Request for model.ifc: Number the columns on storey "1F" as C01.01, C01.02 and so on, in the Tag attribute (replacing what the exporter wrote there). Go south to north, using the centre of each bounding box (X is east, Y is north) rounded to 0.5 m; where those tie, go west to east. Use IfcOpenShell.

First a look at what the model holds.

```python
import ifcopenshell
import ifcopenshell.util.element
import ifcopenshell.util.placement

model = ifcopenshell.open("model.ifc")
print(model.schema)
storey = next(s for s in model.by_type("IfcBuildingStorey") if s.Name == "1F")
columns = [e for e in ifcopenshell.util.element.get_decomposition(storey) if e.is_a("IfcColumn")]
for e in sorted(columns, key=lambda e: e.id()):
    origin = ifcopenshell.util.placement.get_local_placement(e.ObjectPlacement)[:3, 3]
    print(e.id(), e.Tag, e.Name, origin.round(2) + 0.0, sep=" | ")
```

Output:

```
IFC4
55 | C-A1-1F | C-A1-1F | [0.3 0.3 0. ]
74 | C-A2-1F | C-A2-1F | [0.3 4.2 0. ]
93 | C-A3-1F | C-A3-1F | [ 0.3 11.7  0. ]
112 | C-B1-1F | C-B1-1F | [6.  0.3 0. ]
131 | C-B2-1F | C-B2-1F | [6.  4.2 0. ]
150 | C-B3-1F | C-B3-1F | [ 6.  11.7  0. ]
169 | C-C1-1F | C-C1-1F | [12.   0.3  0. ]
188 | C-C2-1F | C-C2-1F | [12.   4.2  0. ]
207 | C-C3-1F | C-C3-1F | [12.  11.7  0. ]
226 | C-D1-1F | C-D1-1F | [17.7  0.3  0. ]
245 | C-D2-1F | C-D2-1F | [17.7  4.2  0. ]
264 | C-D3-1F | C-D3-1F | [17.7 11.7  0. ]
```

```python
import ifcopenshell
import ifcopenshell.geom
import ifcopenshell.util.element
import ifcopenshell.util.shape

model = ifcopenshell.open("model.ifc")
settings = ifcopenshell.geom.settings()
settings.set("use-world-coords", True)


def centre(element):
    shape = ifcopenshell.geom.create_shape(settings, element)
    return ifcopenshell.util.shape.get_bbox_centroid(shape.geometry)


storey = next(s for s in model.by_type("IfcBuildingStorey") if s.Name == "1F")
columns = [e for e in ifcopenshell.util.element.get_decomposition(storey) if e.is_a("IfcColumn")]

# Insertion points can sit at a corner or the storey origin, so sort by the geometry (in metres).
centres = {e: centre(e) for e in columns}
columns.sort(key=lambda e: (round(centres[e][1] / 0.5), centres[e][0]))

for i, e in enumerate(columns, start=1):
    number = f"C01.{i:02d}"
    e.Tag = number
    print(e.id(), number)

model.write("model_v2.ifc")
```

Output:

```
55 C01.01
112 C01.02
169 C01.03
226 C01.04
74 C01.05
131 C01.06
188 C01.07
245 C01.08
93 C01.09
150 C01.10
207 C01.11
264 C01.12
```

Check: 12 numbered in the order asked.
